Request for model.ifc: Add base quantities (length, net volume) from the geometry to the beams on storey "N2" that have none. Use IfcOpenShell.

First a look at what the model holds.

```python
import ifcopenshell
import ifcopenshell.util.element
import ifcopenshell.util.unit

model = ifcopenshell.open("model.ifc")
print(model.schema)
for unit_type in ("LENGTHUNIT", "AREAUNIT", "VOLUMEUNIT"):
    print(unit_type, ifcopenshell.util.unit.calculate_unit_scale(model, unit_type))
storey = next(s for s in model.by_type("IfcBuildingStorey") if s.Name == "N2")
beams = [e for e in ifcopenshell.util.element.get_decomposition(storey) if e.is_a("IfcBeam")]
for e in sorted(beams, key=lambda e: e.id()):
    print(e.id(), e.is_a(), e.Name, list(ifcopenshell.util.element.get_psets(e, qtos_only=True)), sep=" | ")
```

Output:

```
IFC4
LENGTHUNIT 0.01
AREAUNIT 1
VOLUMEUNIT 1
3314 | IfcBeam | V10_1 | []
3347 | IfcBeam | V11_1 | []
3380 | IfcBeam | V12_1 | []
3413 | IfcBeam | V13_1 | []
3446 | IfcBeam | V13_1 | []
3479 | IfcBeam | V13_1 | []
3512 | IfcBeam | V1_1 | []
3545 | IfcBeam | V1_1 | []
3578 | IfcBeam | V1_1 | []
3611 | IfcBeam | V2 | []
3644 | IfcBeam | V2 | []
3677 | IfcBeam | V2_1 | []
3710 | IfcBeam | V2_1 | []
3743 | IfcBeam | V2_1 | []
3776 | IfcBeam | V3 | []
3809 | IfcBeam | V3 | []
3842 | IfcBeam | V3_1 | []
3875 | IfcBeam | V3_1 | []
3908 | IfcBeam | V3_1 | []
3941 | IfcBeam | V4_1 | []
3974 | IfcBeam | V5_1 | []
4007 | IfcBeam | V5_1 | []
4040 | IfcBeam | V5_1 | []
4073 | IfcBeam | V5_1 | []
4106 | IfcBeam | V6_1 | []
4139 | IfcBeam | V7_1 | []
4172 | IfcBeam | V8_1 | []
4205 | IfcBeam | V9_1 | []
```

```python
import ifcopenshell
import ifcopenshell.api.pset
import ifcopenshell.geom
import ifcopenshell.util.element
import ifcopenshell.util.shape
import ifcopenshell.util.unit

model = ifcopenshell.open("model.ifc")
unit_scale = ifcopenshell.util.unit.calculate_unit_scale(model)
volume_scale = ifcopenshell.util.unit.calculate_unit_scale(model, "VOLUMEUNIT")
settings = ifcopenshell.geom.settings()

storey = next(s for s in model.by_type("IfcBuildingStorey") if s.Name == "N2")
beams = [e for e in ifcopenshell.util.element.get_decomposition(storey) if e.is_a("IfcBeam")]

for e in sorted(beams, key=lambda e: e.id()):
    if ifcopenshell.util.element.get_psets(e, qtos_only=True, should_inherit=False):
        continue
    # Geometry comes back in metres, in the element's own axes.
    shape = ifcopenshell.geom.create_shape(settings, e)
    values = {
        "Length": ifcopenshell.util.shape.get_max_xyz(shape.geometry) / unit_scale,
        "NetVolume": ifcopenshell.util.shape.get_volume(shape.geometry) / volume_scale,
    }
    qto = ifcopenshell.api.pset.add_qto(model, product=e, name="Qto_BeamBaseQuantities")
    ifcopenshell.api.pset.edit_qto(model, qto=qto, properties=values)
    print(e.id(), {k: round(v, 3) for k, v in values.items()})

model.write("model_rev.ifc")
```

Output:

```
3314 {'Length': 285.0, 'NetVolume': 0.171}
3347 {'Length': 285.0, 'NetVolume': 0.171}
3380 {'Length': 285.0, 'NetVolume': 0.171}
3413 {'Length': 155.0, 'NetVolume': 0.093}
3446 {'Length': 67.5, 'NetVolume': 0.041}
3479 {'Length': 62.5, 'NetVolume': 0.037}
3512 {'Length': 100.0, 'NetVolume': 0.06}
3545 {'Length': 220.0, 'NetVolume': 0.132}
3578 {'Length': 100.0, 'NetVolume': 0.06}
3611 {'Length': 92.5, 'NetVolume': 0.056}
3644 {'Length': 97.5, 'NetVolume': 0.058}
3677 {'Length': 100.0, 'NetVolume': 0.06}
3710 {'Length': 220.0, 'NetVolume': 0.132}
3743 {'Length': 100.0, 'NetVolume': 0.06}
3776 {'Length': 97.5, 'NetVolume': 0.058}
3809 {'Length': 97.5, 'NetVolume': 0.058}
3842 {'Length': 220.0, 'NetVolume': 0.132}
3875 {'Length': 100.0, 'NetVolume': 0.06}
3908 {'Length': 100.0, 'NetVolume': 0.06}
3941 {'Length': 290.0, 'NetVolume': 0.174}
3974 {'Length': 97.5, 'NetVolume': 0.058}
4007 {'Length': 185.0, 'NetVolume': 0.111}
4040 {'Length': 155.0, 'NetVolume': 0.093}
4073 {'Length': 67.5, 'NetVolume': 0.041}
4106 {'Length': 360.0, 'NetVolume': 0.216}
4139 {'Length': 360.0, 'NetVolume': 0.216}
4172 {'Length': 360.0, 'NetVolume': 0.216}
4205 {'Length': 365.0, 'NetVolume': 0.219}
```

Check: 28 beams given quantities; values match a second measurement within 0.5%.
